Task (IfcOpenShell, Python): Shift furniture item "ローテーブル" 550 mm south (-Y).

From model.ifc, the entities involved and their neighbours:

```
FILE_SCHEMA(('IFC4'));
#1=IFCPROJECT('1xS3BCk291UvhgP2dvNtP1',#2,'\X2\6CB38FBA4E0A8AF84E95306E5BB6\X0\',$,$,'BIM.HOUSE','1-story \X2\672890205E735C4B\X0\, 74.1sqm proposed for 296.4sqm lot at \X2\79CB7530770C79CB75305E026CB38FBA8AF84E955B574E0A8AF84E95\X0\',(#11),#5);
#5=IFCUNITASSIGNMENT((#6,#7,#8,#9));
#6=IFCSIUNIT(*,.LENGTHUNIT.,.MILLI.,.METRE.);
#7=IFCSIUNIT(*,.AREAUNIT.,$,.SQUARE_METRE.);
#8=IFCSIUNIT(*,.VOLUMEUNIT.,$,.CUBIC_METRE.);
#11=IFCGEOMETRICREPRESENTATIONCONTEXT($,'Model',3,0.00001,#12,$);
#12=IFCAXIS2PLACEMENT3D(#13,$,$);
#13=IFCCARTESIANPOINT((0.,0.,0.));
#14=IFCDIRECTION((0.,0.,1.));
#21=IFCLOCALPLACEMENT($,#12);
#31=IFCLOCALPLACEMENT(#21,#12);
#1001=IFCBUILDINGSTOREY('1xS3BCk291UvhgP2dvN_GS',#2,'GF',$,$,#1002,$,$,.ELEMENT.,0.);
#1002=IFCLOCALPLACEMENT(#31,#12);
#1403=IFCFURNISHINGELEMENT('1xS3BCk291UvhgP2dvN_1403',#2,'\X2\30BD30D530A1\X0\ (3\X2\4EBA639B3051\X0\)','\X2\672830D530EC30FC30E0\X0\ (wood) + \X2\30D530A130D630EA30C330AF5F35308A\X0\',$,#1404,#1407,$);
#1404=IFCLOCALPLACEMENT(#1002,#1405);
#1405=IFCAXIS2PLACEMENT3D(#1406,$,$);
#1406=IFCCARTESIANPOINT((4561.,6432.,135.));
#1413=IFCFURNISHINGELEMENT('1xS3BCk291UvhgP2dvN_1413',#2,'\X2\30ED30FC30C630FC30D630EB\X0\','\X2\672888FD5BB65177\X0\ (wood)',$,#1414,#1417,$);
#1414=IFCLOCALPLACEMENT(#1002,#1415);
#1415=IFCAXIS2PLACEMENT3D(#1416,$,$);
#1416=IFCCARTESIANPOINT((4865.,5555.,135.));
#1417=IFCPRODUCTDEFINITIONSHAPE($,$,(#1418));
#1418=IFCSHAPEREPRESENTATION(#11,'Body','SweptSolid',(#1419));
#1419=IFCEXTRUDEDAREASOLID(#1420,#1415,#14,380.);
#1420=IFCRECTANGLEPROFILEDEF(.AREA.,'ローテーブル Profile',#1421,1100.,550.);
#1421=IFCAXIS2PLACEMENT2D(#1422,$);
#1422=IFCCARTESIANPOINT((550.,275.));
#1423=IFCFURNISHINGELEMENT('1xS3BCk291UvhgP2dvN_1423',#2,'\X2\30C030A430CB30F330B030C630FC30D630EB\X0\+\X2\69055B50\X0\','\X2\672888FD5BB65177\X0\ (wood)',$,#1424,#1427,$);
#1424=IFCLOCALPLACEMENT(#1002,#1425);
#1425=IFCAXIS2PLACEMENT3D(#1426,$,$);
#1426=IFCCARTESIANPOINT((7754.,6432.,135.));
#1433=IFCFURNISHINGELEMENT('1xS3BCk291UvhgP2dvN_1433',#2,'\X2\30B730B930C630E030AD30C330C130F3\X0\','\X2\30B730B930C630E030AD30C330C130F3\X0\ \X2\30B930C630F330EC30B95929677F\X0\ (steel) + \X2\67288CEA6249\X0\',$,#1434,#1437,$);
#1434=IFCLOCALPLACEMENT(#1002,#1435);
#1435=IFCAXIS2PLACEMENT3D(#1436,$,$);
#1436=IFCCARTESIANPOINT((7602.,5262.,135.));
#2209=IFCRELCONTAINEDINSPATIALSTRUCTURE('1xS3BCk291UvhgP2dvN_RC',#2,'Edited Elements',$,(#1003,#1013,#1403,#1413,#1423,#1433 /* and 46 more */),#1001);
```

```python
import ifcopenshell
import ifcopenshell.api.geometry
import ifcopenshell.util.placement
import ifcopenshell.util.unit

model = ifcopenshell.open("model.ifc")
unit_scale = ifcopenshell.util.unit.calculate_unit_scale(model)

item = model.by_id(1413)
matrix = ifcopenshell.util.placement.get_local_placement(item.ObjectPlacement)
matrix[1, 3] -= 0.55 / unit_scale
ifcopenshell.api.geometry.edit_object_placement(model, product=item, matrix=matrix, is_si=False)

print(ifcopenshell.util.placement.get_local_placement(item.ObjectPlacement).round(3) + 0.0)

model.write("model_rev.ifc")
```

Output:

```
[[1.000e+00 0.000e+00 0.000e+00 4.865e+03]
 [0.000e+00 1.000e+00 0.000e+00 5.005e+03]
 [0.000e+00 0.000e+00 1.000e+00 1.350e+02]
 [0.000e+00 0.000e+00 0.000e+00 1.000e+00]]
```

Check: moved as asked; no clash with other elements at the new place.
